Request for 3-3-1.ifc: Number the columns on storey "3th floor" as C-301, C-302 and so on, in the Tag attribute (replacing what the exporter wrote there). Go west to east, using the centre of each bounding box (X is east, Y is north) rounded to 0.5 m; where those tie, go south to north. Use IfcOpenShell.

First a look at what the model holds.

```python
import ifcopenshell
import ifcopenshell.util.element
import ifcopenshell.util.placement

model = ifcopenshell.open("3-3-1.ifc")
print(model.schema)
storey = next(s for s in model.by_type("IfcBuildingStorey") if s.Name == "3th floor")
columns = [e for e in ifcopenshell.util.element.get_decomposition(storey) if e.is_a("IfcColumn")]
for e in sorted(columns, key=lambda e: e.id()):
    origin = ifcopenshell.util.placement.get_local_placement(e.ObjectPlacement)[:3, 3]
    print(e.id(), e.Tag, e.Name, origin.round(2) + 0.0, sep=" | ")
```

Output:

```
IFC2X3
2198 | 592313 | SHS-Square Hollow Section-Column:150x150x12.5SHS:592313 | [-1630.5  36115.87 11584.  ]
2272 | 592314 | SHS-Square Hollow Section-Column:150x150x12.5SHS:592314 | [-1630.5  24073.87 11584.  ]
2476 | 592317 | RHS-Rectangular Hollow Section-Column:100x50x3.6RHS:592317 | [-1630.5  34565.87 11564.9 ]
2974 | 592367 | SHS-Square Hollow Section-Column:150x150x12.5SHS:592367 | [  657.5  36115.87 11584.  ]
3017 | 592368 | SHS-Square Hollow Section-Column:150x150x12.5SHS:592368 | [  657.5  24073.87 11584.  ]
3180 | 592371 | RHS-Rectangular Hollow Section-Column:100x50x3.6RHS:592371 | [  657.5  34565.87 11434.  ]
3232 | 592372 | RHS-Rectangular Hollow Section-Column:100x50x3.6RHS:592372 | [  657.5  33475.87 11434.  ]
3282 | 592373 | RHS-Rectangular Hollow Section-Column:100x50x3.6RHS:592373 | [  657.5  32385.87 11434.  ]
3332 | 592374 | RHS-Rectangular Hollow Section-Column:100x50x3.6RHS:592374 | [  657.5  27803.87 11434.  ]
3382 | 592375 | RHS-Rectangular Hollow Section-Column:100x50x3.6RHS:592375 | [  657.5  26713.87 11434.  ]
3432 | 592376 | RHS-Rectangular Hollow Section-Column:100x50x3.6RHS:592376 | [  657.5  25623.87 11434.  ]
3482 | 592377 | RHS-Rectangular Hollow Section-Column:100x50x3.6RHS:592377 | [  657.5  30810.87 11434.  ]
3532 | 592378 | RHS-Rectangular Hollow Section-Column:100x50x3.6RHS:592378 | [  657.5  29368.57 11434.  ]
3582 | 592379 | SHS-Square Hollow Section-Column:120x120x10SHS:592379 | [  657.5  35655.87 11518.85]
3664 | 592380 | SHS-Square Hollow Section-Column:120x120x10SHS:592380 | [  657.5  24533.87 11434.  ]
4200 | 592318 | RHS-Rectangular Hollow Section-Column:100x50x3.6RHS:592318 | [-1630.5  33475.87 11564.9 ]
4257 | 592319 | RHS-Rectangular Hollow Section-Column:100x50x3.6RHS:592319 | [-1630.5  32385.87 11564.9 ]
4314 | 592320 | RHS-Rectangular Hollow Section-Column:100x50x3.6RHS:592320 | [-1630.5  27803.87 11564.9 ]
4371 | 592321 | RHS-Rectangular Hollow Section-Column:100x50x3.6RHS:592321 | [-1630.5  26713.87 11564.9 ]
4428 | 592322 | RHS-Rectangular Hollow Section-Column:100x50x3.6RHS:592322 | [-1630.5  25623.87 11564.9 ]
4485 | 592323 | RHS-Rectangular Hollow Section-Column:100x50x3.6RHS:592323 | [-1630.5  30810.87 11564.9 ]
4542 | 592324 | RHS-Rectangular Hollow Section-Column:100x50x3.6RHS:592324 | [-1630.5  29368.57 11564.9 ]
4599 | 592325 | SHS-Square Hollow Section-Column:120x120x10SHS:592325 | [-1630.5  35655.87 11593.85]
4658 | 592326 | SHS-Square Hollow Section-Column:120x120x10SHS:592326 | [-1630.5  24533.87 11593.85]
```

```python
import ifcopenshell
import ifcopenshell.geom
import ifcopenshell.util.element
import ifcopenshell.util.shape

model = ifcopenshell.open("3-3-1.ifc")
settings = ifcopenshell.geom.settings()
settings.set("use-world-coords", True)


def centre(element):
    shape = ifcopenshell.geom.create_shape(settings, element)
    return ifcopenshell.util.shape.get_bbox_centroid(shape.geometry)


storey = next(s for s in model.by_type("IfcBuildingStorey") if s.Name == "3th floor")
columns = [e for e in ifcopenshell.util.element.get_decomposition(storey) if e.is_a("IfcColumn")]

# Insertion points can sit at a corner or the storey origin, so sort by the geometry (in metres).
centres = {e: centre(e) for e in columns}
columns.sort(key=lambda e: (round(centres[e][0] / 0.5), centres[e][1]))

for i, e in enumerate(columns, start=1):
    number = f"C-3{i:02d}"
    e.Tag = number
    print(e.id(), number)

model.write("3-3-1-out.ifc")
```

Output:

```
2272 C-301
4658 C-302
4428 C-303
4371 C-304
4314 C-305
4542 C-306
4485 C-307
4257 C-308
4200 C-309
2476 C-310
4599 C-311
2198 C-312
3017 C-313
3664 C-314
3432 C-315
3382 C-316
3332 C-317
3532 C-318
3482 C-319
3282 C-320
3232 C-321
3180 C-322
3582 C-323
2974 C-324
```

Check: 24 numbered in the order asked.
